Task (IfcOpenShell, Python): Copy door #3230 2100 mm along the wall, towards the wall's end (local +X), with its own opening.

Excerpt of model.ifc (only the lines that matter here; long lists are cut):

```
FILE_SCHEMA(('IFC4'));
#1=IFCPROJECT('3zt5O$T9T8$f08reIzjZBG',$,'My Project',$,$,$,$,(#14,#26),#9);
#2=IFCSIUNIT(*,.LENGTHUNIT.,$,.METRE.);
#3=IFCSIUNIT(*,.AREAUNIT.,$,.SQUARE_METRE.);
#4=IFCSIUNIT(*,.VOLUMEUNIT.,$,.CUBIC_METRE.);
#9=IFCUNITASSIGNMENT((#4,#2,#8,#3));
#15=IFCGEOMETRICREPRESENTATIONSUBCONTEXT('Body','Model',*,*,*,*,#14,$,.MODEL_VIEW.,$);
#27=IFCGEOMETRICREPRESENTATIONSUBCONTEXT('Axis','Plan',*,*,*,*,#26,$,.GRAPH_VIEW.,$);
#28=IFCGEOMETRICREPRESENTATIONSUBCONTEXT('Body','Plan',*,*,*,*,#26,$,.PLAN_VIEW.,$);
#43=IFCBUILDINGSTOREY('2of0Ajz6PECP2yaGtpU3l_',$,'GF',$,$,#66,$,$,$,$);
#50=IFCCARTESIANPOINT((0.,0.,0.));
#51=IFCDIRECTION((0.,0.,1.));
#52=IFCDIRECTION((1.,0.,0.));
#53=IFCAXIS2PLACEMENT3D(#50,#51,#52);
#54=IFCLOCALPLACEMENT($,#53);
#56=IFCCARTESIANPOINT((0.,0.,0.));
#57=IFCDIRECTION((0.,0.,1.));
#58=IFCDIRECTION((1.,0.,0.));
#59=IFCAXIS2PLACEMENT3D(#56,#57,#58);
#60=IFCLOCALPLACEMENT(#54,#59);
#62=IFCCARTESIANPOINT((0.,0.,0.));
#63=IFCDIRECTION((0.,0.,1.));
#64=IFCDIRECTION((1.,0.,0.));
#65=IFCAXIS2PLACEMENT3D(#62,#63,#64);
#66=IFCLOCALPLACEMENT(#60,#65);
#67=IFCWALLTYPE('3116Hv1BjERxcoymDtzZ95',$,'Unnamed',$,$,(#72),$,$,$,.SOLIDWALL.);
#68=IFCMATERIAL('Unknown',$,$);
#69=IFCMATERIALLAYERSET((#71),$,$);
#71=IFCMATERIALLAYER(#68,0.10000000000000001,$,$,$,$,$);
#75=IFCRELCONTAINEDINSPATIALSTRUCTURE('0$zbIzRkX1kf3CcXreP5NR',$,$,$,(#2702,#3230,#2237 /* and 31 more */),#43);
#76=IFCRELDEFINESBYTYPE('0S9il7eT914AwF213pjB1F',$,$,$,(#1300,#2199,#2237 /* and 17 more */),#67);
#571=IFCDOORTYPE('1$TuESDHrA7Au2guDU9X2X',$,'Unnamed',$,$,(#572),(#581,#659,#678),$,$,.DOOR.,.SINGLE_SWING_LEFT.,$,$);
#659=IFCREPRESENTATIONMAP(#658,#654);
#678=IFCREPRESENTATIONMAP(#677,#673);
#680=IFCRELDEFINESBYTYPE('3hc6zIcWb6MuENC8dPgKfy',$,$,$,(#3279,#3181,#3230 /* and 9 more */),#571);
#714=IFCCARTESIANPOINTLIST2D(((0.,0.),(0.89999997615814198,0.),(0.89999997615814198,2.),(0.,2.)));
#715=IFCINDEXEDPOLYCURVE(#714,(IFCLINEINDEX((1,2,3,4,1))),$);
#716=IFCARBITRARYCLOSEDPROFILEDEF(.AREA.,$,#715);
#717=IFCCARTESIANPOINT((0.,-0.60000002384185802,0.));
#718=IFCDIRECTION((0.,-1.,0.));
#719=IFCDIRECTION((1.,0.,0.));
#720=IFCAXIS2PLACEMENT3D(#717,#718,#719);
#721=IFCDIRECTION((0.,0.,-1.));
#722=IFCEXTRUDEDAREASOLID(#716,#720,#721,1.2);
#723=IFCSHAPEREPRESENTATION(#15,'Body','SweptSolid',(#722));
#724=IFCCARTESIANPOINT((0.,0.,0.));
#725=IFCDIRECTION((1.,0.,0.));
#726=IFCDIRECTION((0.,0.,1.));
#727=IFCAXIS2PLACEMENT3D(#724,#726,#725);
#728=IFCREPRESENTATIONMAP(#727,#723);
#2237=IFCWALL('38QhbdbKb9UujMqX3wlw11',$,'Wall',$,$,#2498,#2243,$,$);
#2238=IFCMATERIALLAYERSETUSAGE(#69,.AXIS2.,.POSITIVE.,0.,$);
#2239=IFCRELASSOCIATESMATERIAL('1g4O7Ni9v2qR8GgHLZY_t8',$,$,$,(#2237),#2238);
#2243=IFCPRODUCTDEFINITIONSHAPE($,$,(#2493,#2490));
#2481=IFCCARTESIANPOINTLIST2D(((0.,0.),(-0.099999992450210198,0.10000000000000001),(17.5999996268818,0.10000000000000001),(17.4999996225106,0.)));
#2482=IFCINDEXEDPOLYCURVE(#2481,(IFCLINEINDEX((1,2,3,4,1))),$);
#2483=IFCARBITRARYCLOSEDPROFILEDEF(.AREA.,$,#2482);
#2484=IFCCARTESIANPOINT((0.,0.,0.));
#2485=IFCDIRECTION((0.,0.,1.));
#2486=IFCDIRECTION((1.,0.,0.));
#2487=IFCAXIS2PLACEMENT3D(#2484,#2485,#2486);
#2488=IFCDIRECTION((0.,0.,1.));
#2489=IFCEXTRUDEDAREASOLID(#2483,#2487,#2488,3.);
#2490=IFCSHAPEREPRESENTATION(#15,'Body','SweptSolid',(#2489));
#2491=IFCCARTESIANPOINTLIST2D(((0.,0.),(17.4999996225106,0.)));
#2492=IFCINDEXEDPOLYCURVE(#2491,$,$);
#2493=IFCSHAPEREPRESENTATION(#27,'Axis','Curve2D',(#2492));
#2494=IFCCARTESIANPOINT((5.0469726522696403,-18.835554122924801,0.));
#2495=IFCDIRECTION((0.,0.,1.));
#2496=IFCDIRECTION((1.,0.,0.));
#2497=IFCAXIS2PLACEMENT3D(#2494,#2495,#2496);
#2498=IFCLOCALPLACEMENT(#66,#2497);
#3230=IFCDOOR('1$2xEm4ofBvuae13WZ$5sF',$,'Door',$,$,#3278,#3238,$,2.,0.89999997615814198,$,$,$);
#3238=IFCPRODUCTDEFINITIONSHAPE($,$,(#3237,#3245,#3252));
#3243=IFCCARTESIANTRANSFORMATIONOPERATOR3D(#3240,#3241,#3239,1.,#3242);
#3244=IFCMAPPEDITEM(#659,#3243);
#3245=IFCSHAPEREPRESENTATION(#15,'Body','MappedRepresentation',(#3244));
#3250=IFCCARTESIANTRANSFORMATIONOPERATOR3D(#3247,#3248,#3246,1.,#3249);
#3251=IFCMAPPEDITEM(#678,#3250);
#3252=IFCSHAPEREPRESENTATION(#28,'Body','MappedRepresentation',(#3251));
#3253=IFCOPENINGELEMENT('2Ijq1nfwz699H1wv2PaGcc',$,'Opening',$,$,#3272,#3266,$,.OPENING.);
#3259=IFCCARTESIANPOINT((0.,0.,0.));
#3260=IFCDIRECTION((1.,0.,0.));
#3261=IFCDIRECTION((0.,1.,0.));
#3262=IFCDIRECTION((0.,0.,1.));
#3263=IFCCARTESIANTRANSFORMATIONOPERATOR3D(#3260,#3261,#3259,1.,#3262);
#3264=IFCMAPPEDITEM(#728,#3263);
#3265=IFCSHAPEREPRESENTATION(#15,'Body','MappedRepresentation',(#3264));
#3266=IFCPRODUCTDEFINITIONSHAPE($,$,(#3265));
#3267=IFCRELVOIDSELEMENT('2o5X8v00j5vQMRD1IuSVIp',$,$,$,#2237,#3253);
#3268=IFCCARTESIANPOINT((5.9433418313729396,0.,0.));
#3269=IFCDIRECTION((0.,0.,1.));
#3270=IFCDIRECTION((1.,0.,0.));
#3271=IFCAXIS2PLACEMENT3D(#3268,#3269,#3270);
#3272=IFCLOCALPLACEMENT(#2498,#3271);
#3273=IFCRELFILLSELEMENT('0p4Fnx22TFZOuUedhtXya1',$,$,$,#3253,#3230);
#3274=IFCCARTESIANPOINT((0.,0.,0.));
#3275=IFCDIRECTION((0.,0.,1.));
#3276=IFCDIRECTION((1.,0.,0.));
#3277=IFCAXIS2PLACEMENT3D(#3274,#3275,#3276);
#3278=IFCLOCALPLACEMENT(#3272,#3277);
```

```python
import ifcopenshell
import ifcopenshell.api.feature
import ifcopenshell.api.geometry
import ifcopenshell.api.root
import ifcopenshell.geom
import ifcopenshell.util.element
import ifcopenshell.util.placement
import ifcopenshell.util.shape
import ifcopenshell.util.unit

model = ifcopenshell.open("model.ifc")
unit_scale = ifcopenshell.util.unit.calculate_unit_scale(model)
settings = ifcopenshell.geom.settings()


def volume(element):
    """Net volume in cubic metres, openings subtracted."""
    shape = ifcopenshell.geom.create_shape(settings, element)
    return ifcopenshell.util.shape.get_volume(shape.geometry)


door = model.by_guid("1$2xEm4ofBvuae13WZ$5sF")
opening = door.FillsVoids[0].RelatingOpeningElement
wall = opening.VoidsElements[0].RelatingBuildingElement
before = volume(wall)
shift = ifcopenshell.util.placement.get_local_placement(wall.ObjectPlacement)[:3, 0] * 2.1 / unit_scale

# copy_class copies the void relationship, type, container and properties, but no geometry.
new_opening = ifcopenshell.api.root.copy_class(model, product=opening)
new_opening.Representation = ifcopenshell.util.element.copy_deep(
    model, opening.Representation, exclude=["IfcGeometricRepresentationContext", "IfcRepresentationMap"]
)
new_door = ifcopenshell.api.root.copy_class(model, product=door)
new_door.Representation = ifcopenshell.util.element.copy_deep(
    model, door.Representation, exclude=["IfcGeometricRepresentationContext", "IfcRepresentationMap"]
)
ifcopenshell.api.feature.add_filling(model, opening=new_opening, element=new_door)

for old, new in ((opening, new_opening), (door, new_door)):
    matrix = ifcopenshell.util.placement.get_local_placement(old.ObjectPlacement)
    matrix[:3, 3] += shift
    ifcopenshell.api.geometry.edit_object_placement(model, product=new, matrix=matrix, is_si=False)

after = volume(wall)

print(f"wall volume {before:.3f} -> {after:.3f} m3")

model.write("model_edited.ifc")
```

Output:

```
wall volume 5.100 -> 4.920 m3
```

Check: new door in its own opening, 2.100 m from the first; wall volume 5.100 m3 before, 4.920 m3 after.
